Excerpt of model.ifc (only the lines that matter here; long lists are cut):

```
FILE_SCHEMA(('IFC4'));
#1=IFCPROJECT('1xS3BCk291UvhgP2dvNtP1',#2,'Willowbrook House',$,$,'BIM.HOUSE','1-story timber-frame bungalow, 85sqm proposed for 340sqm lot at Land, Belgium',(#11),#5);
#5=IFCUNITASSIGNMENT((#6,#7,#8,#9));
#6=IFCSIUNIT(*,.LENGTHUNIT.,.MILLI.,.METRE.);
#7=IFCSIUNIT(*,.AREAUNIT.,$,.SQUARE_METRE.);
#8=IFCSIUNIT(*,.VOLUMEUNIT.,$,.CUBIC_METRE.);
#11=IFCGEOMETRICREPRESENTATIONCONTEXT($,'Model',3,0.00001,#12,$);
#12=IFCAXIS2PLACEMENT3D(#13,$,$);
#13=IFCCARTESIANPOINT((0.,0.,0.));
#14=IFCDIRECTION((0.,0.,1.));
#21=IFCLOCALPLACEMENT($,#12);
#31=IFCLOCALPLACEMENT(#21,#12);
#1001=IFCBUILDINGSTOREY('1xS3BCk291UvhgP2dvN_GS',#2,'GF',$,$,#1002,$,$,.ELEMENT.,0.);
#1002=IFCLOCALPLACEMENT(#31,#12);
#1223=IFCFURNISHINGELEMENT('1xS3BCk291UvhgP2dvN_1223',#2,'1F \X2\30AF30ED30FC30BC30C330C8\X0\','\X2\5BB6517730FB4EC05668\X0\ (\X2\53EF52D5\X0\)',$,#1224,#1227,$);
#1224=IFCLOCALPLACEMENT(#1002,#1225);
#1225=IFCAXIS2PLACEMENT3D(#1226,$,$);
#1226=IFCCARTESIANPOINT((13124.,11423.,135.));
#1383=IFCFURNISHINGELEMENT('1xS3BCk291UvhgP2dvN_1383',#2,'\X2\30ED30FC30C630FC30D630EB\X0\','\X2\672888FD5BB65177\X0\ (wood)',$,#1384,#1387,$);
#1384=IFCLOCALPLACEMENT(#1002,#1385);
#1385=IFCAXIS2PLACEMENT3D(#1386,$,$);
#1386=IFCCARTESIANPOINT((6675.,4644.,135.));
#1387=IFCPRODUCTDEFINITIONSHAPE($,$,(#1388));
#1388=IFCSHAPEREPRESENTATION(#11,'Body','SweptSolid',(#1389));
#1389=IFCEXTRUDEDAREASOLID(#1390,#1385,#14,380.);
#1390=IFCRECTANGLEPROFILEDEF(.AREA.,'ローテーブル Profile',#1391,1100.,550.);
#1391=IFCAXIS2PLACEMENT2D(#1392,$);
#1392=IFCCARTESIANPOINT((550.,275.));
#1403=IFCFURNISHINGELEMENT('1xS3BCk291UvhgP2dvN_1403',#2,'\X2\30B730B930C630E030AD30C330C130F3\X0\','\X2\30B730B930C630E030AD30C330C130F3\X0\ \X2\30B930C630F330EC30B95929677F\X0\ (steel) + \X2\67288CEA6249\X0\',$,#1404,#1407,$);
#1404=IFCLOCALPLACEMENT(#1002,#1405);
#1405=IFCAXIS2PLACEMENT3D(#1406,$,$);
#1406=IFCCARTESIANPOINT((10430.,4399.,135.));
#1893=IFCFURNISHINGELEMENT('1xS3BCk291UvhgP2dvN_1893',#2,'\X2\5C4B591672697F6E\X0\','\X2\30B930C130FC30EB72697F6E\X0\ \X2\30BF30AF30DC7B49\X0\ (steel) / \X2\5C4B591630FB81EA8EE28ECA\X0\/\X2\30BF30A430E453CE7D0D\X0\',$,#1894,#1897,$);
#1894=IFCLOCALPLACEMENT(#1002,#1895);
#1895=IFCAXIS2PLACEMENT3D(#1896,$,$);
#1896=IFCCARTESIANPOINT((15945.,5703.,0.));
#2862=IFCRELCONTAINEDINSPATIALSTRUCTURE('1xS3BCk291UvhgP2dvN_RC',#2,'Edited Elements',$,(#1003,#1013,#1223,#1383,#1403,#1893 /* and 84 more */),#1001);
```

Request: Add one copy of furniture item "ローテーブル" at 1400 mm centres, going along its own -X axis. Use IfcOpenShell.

```python
import ifcopenshell
import ifcopenshell.api.geometry
import ifcopenshell.api.root
import ifcopenshell.util.element
import ifcopenshell.util.placement
import ifcopenshell.util.unit

model = ifcopenshell.open("model.ifc")
unit_scale = ifcopenshell.util.unit.calculate_unit_scale(model)


def reuse_history(source, copy):
    """copy_class also copies each property set's owner history, people and application; keep the originals."""
    for rel in copy.IsDefinedBy:
        if rel.is_a("IfcRelDefinesByProperties") and (history := rel.RelatingPropertyDefinition.OwnerHistory):
            rel.RelatingPropertyDefinition.OwnerHistory = source.OwnerHistory
            ifcopenshell.util.element.remove_deep2(model, history)


source = model.by_guid("1xS3BCk291UvhgP2dvN_1383")
base = ifcopenshell.util.placement.get_local_placement(source.ObjectPlacement)
step = -base[:3, 0] * 1.4 / unit_scale

for i in range(1, 2):
    copy = ifcopenshell.api.root.copy_class(model, product=source)
    copy.Representation = ifcopenshell.util.element.copy_deep(
        model, source.Representation, exclude=["IfcGeometricRepresentationContext", "IfcRepresentationMap"]
    )
    reuse_history(source, copy)
    matrix = base.copy()
    matrix[:3, 3] += i * step
    print("added at", matrix[:3, 3].round(3) + 0.0)
    ifcopenshell.api.geometry.edit_object_placement(model, product=copy, matrix=matrix, is_si=False)

model.write("model_v2.ifc")
```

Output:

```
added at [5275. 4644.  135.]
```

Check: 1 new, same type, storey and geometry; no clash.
